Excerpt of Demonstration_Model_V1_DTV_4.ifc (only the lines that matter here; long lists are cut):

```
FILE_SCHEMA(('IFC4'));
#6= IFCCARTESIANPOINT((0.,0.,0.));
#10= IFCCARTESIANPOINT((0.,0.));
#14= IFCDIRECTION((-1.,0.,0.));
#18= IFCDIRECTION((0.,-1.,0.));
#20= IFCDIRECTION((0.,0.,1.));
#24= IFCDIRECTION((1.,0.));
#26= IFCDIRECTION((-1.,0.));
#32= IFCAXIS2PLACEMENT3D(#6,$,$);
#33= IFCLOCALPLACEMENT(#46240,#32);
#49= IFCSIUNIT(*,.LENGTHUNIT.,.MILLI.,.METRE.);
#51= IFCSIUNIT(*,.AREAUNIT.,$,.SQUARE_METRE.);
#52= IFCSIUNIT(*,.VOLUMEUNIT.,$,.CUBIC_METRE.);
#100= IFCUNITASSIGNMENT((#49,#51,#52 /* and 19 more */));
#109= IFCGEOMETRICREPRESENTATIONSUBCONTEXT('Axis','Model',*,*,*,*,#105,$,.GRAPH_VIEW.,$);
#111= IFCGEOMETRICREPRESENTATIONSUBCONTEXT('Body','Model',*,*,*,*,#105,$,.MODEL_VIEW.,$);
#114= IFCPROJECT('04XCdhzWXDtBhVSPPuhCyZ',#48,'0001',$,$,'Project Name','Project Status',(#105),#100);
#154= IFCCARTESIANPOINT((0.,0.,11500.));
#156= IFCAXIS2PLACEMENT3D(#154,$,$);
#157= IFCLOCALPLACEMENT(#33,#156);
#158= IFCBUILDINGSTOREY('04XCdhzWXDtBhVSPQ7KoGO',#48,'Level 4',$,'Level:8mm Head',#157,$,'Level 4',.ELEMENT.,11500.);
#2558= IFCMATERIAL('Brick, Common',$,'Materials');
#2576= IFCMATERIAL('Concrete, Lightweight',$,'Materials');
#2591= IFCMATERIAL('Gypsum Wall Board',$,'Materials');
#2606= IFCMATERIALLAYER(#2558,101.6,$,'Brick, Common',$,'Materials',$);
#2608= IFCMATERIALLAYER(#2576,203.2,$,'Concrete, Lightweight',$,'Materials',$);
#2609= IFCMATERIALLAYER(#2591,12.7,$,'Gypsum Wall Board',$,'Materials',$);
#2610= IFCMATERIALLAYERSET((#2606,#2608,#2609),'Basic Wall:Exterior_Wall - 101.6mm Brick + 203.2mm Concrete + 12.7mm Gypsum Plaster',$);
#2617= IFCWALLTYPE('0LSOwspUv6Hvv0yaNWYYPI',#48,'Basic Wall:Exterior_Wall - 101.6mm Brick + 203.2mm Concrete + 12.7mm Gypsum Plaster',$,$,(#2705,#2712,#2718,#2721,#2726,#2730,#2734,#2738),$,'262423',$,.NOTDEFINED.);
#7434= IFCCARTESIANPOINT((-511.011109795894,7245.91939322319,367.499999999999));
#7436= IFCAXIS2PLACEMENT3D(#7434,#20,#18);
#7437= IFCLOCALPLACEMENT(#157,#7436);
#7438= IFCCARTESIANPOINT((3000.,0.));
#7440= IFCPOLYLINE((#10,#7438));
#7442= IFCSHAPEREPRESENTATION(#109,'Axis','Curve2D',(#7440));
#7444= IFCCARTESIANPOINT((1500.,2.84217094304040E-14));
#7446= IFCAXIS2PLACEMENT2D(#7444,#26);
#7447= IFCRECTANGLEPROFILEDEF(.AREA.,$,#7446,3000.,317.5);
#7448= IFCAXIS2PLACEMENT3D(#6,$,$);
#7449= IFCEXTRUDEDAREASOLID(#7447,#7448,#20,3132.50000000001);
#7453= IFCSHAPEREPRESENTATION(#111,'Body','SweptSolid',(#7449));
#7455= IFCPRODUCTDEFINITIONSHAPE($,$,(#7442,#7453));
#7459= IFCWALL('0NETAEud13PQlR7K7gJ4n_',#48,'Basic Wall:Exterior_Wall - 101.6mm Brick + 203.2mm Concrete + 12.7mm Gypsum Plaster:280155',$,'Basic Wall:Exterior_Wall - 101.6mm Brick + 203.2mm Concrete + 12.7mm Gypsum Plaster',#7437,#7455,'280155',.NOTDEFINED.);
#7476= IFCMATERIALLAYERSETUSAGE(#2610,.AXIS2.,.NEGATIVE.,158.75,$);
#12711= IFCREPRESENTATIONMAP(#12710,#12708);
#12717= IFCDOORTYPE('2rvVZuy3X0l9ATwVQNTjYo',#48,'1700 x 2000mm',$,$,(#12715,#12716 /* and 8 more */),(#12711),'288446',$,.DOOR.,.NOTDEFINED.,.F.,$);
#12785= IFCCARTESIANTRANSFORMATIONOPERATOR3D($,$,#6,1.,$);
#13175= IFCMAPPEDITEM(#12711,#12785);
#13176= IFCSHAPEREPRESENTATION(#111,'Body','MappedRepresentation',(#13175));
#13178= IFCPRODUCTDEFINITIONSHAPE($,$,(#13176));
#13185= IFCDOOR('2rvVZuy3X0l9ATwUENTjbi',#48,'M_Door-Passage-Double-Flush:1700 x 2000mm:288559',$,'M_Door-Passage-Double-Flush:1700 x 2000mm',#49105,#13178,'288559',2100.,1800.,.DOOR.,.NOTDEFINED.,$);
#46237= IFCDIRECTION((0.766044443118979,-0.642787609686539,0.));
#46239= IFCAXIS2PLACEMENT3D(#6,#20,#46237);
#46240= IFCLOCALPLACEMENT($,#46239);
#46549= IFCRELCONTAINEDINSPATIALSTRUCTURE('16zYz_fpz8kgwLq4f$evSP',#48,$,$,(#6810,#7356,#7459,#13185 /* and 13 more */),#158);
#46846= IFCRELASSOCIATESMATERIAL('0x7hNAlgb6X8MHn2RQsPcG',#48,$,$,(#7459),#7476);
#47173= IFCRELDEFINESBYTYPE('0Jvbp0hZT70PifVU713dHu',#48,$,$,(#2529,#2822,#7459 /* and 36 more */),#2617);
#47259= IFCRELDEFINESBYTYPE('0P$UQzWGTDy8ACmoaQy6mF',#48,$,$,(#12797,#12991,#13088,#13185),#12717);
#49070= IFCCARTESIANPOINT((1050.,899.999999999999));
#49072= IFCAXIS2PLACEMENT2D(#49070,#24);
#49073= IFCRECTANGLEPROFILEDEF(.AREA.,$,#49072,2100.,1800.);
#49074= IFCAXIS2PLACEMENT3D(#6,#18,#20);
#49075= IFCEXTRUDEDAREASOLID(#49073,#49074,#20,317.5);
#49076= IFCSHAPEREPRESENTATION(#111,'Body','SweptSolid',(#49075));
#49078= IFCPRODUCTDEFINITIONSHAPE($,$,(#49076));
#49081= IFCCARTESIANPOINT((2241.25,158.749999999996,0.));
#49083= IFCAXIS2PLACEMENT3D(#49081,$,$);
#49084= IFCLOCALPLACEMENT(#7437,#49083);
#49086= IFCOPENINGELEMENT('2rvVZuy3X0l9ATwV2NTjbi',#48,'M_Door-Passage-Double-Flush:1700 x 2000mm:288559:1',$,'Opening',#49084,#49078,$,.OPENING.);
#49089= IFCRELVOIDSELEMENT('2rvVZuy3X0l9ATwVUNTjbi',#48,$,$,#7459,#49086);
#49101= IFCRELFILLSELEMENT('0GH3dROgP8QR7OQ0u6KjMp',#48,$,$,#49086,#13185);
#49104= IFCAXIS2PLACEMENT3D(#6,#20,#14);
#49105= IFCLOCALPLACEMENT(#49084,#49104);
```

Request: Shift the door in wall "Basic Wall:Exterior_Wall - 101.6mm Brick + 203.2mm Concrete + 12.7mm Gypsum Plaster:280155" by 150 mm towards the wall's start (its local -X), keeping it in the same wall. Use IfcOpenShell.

```python
import ifcopenshell
import ifcopenshell.api.geometry
import ifcopenshell.util.placement
import ifcopenshell.util.unit

model = ifcopenshell.open("Demonstration_Model_V1_DTV_4.ifc")
unit_scale = ifcopenshell.util.unit.calculate_unit_scale(model)

door = model.by_id(13185)
opening = door.FillsVoids[0].RelatingOpeningElement
wall = opening.VoidsElements[0].RelatingBuildingElement

wall_matrix = ifcopenshell.util.placement.get_local_placement(wall.ObjectPlacement)
shift = wall_matrix[:3, 0] * -0.15 / unit_scale
before = ifcopenshell.util.placement.get_local_placement(door.ObjectPlacement)[:3, 3].copy()

# The door is placed relative to its opening, so it follows when the opening moves.
matrix = ifcopenshell.util.placement.get_local_placement(opening.ObjectPlacement)
matrix[:3, 3] += shift
ifcopenshell.api.geometry.edit_object_placement(
    model, product=opening, matrix=matrix, is_si=False, should_transform_children=True
)

after = ifcopenshell.util.placement.get_local_placement(door.ObjectPlacement)[:3, 3]
print("door moved by", (after - before).round(3) + 0.0)

model.write("Demonstration_Model_V1_DTV_4_v2.ifc")
```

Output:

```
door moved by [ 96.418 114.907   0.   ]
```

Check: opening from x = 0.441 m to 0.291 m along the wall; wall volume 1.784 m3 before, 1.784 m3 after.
